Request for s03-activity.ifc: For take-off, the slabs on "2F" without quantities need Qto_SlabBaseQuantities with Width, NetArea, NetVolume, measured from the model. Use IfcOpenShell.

First a look at what the model holds.

```python
import ifcopenshell
import ifcopenshell.util.element
import ifcopenshell.util.unit

model = ifcopenshell.open("s03-activity.ifc")
print(model.schema)
for unit_type in ("LENGTHUNIT", "AREAUNIT", "VOLUMEUNIT"):
    print(unit_type, ifcopenshell.util.unit.calculate_unit_scale(model, unit_type))
storey = next(s for s in model.by_type("IfcBuildingStorey") if s.Name == "2F")
slabs = [e for e in ifcopenshell.util.element.get_decomposition(storey) if e.is_a("IfcSlab")]
for e in sorted(slabs, key=lambda e: e.id()):
    print(e.id(), e.is_a(), e.Name, list(ifcopenshell.util.element.get_psets(e, qtos_only=True)), sep=" | ")
```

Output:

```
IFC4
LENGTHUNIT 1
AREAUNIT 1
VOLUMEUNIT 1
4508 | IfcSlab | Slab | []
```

```python
import ifcopenshell
import ifcopenshell.api.pset
import ifcopenshell.geom
import ifcopenshell.util.element
import ifcopenshell.util.shape
import ifcopenshell.util.unit

model = ifcopenshell.open("s03-activity.ifc")
unit_scale = ifcopenshell.util.unit.calculate_unit_scale(model)
area_scale = ifcopenshell.util.unit.calculate_unit_scale(model, "AREAUNIT")
volume_scale = ifcopenshell.util.unit.calculate_unit_scale(model, "VOLUMEUNIT")
settings = ifcopenshell.geom.settings()

storey = next(s for s in model.by_type("IfcBuildingStorey") if s.Name == "2F")
slabs = [e for e in ifcopenshell.util.element.get_decomposition(storey) if e.is_a("IfcSlab")]

for e in sorted(slabs, key=lambda e: e.id()):
    if ifcopenshell.util.element.get_psets(e, qtos_only=True, should_inherit=False):
        continue
    # Geometry comes back in metres, in the element's own axes.
    shape = ifcopenshell.geom.create_shape(settings, e)
    values = {
        "Width": ifcopenshell.util.shape.get_z(shape.geometry) / unit_scale,
        "NetArea": ifcopenshell.util.shape.get_footprint_area(shape.geometry) / area_scale,
        "NetVolume": ifcopenshell.util.shape.get_volume(shape.geometry) / volume_scale,
    }
    qto = ifcopenshell.api.pset.add_qto(model, product=e, name="Qto_SlabBaseQuantities")
    ifcopenshell.api.pset.edit_qto(model, qto=qto, properties=values)
    print(e.id(), {k: round(v, 3) for k, v in values.items()})

model.write("s03-activity-out.ifc")
```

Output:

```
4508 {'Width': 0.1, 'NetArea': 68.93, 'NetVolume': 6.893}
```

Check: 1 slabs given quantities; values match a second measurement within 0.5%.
